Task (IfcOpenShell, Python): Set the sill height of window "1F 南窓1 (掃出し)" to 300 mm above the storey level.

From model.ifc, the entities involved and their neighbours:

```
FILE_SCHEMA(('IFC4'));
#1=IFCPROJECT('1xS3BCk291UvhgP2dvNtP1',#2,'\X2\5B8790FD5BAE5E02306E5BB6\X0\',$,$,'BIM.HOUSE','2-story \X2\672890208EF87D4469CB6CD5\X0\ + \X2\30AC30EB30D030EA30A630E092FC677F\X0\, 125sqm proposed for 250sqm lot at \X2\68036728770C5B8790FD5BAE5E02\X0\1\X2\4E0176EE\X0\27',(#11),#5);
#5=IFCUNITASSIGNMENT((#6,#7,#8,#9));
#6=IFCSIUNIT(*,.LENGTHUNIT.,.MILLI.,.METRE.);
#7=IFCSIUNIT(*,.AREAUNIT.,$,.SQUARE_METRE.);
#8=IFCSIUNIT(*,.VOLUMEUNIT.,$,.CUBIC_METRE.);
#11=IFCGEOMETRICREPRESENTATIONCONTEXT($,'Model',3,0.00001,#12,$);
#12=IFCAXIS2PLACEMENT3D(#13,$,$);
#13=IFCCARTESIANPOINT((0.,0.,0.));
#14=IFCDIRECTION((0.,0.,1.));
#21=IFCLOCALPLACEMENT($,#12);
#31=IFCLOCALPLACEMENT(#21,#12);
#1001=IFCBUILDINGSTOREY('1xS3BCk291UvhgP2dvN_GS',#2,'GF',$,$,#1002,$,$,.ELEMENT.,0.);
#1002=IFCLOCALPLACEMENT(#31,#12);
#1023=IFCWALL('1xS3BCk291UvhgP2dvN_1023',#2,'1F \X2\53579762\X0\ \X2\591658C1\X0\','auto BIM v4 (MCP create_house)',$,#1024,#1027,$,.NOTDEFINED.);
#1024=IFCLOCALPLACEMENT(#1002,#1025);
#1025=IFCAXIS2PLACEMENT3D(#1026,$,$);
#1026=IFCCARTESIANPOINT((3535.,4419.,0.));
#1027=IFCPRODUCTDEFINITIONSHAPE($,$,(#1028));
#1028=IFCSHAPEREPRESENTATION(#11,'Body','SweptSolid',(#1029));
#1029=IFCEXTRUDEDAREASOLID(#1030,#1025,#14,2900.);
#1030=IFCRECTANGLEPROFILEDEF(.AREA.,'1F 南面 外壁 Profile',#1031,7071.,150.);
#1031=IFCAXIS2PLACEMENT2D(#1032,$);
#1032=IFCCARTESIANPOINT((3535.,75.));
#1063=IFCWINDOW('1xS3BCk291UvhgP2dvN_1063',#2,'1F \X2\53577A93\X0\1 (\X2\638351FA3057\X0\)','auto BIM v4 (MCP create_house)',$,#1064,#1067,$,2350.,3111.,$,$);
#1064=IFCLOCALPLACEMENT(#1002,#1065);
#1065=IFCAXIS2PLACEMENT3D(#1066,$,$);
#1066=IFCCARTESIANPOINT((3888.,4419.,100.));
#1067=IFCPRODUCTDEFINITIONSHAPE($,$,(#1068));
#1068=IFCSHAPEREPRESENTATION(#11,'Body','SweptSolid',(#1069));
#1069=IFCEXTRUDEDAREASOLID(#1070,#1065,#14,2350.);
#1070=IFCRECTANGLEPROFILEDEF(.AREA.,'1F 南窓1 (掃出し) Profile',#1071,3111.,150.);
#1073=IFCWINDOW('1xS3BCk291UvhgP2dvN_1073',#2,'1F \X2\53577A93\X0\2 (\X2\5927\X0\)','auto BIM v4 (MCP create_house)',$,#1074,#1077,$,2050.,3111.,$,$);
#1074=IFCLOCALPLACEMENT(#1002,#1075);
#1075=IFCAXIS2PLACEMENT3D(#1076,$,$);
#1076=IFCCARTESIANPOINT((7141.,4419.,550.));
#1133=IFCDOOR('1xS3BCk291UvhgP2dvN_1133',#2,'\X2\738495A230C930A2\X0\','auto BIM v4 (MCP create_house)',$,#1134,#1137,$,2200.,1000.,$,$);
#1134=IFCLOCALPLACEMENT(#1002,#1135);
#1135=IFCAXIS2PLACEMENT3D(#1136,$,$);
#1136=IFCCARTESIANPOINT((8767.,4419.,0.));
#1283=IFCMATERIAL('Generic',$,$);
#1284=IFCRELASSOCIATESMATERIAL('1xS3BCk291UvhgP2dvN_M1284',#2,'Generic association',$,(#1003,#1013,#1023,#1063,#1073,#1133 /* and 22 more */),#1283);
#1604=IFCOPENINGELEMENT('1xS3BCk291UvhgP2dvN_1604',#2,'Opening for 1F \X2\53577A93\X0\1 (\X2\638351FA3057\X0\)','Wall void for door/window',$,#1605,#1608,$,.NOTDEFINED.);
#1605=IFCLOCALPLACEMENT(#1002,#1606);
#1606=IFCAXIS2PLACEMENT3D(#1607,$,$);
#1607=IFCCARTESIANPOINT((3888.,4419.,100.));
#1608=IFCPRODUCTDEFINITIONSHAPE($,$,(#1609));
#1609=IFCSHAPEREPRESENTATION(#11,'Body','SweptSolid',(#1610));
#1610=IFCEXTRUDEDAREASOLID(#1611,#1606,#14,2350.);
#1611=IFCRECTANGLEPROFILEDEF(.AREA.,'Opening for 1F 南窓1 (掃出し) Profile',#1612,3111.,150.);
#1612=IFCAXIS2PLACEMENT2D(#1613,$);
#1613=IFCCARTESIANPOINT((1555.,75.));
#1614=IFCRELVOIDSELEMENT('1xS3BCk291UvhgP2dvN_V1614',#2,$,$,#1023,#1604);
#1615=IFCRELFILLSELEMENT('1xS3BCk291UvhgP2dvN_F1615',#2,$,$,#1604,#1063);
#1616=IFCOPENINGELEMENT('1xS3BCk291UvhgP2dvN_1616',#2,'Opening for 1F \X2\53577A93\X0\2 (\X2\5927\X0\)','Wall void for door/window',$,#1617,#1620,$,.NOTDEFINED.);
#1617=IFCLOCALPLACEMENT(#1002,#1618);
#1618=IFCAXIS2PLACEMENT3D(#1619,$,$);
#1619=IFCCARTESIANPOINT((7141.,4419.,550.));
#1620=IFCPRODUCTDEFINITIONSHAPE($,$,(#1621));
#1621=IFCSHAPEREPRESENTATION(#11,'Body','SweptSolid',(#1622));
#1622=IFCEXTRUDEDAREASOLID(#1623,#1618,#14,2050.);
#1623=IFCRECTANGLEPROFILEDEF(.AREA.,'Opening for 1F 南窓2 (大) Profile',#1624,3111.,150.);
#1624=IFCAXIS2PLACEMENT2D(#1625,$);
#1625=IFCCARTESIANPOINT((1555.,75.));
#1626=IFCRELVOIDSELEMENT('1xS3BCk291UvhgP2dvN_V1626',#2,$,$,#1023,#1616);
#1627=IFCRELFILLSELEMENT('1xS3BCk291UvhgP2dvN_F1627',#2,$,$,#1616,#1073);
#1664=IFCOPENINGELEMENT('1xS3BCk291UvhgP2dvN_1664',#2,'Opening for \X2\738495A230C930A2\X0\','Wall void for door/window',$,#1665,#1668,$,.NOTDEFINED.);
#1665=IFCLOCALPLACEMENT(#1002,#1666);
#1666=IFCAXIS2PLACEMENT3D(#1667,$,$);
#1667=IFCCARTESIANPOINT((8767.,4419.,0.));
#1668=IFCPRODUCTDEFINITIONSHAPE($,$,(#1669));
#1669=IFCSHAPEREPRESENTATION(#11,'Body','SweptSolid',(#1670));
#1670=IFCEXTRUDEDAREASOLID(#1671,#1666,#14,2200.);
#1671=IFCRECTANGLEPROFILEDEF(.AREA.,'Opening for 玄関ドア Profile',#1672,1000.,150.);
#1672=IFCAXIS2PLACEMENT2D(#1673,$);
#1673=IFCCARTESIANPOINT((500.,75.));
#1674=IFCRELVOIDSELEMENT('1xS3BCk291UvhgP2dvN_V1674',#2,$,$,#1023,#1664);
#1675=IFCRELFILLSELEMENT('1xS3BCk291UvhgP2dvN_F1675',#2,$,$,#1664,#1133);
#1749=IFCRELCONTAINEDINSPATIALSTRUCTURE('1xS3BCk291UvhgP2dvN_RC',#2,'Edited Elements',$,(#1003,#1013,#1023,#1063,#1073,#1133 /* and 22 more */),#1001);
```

```python
import numpy as np
import ifcopenshell
import ifcopenshell.api.geometry
import ifcopenshell.geom
import ifcopenshell.util.element
import ifcopenshell.util.placement
import ifcopenshell.util.shape
import ifcopenshell.util.unit

model = ifcopenshell.open("model.ifc")
unit_scale = ifcopenshell.util.unit.calculate_unit_scale(model)

window = model.by_id(1063)
opening = window.FillsVoids[0].RelatingOpeningElement
storey = ifcopenshell.util.element.get_container(window, ifc_class="IfcBuildingStorey")
level = ifcopenshell.util.placement.get_local_placement(storey.ObjectPlacement)[2, 3]

# The opening's origin need not be at the sill, so measure its lowest point.
shape = ifcopenshell.geom.create_shape(ifcopenshell.geom.settings(), opening)
bottom = ifcopenshell.util.shape.get_shape_bottom_elevation(shape, shape.geometry) / unit_scale
dz = level + 300.0 - bottom

shift = np.array([0.0, 0.0, dz])
# The window is not placed relative to its opening, so move both.
for product in (opening, window):
    matrix = ifcopenshell.util.placement.get_local_placement(product.ObjectPlacement)
    matrix[:3, 3] += shift
    ifcopenshell.api.geometry.edit_object_placement(model, product=product, matrix=matrix, is_si=False)

print(f"moved by {dz * unit_scale:+.3f} m")

model.write("model-out.ifc")
```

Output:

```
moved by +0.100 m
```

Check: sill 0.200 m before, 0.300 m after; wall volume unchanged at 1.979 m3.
